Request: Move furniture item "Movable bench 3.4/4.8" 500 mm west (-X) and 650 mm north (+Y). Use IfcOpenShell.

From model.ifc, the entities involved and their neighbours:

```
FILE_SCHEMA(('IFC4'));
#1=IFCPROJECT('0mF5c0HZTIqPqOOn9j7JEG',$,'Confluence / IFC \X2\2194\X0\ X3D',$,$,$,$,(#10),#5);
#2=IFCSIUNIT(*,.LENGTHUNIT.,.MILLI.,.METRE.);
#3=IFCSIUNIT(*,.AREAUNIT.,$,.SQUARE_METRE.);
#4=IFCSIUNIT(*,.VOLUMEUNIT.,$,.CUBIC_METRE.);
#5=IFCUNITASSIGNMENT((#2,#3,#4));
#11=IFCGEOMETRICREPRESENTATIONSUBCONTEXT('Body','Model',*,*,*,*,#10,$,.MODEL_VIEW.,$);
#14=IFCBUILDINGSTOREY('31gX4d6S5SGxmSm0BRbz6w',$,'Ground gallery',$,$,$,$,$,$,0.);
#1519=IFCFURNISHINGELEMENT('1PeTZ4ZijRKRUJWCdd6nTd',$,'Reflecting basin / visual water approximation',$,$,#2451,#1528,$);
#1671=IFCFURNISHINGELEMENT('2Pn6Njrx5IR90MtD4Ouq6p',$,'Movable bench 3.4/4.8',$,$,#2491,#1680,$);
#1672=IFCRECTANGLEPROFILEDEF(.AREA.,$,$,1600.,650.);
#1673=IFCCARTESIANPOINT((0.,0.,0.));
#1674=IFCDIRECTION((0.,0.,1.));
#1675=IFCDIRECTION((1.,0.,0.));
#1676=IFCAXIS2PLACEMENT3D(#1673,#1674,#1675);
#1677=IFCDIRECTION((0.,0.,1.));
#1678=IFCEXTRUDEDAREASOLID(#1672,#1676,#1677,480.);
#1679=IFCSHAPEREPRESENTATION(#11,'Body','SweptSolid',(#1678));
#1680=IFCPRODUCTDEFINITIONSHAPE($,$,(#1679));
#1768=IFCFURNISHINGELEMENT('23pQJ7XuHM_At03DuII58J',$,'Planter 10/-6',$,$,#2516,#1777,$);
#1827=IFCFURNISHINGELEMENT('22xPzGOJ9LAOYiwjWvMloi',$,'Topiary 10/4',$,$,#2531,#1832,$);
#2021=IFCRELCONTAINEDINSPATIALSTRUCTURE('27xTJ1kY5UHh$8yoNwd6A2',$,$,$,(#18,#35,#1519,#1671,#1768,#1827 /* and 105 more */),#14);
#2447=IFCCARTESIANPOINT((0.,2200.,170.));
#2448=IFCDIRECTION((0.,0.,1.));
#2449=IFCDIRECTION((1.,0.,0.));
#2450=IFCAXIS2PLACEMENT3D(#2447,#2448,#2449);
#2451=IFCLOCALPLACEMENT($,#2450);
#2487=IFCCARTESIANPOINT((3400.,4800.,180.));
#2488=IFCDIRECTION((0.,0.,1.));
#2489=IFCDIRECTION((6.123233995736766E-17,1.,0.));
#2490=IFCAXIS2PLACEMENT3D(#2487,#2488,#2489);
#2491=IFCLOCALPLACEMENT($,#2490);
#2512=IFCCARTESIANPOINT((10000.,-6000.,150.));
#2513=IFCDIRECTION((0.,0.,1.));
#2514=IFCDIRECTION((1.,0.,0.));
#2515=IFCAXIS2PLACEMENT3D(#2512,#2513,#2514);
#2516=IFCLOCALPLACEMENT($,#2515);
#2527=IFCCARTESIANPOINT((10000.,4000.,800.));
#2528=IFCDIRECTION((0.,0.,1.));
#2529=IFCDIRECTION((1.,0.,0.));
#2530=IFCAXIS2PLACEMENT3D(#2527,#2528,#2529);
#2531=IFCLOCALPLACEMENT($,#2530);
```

```python
import ifcopenshell
import ifcopenshell.api.geometry
import ifcopenshell.util.placement
import ifcopenshell.util.unit

model = ifcopenshell.open("model.ifc")
unit_scale = ifcopenshell.util.unit.calculate_unit_scale(model)

item = model.by_id(1671)
matrix = ifcopenshell.util.placement.get_local_placement(item.ObjectPlacement)
matrix[0, 3] -= 0.5 / unit_scale
matrix[1, 3] += 0.65 / unit_scale
ifcopenshell.api.geometry.edit_object_placement(model, product=item, matrix=matrix, is_si=False)

print(ifcopenshell.util.placement.get_local_placement(item.ObjectPlacement).round(3) + 0.0)

model.write("model_edited.ifc")
```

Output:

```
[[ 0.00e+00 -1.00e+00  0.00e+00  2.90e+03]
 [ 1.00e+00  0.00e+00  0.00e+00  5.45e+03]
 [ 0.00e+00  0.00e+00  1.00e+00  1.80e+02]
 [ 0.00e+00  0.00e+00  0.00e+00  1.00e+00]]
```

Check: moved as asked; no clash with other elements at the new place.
